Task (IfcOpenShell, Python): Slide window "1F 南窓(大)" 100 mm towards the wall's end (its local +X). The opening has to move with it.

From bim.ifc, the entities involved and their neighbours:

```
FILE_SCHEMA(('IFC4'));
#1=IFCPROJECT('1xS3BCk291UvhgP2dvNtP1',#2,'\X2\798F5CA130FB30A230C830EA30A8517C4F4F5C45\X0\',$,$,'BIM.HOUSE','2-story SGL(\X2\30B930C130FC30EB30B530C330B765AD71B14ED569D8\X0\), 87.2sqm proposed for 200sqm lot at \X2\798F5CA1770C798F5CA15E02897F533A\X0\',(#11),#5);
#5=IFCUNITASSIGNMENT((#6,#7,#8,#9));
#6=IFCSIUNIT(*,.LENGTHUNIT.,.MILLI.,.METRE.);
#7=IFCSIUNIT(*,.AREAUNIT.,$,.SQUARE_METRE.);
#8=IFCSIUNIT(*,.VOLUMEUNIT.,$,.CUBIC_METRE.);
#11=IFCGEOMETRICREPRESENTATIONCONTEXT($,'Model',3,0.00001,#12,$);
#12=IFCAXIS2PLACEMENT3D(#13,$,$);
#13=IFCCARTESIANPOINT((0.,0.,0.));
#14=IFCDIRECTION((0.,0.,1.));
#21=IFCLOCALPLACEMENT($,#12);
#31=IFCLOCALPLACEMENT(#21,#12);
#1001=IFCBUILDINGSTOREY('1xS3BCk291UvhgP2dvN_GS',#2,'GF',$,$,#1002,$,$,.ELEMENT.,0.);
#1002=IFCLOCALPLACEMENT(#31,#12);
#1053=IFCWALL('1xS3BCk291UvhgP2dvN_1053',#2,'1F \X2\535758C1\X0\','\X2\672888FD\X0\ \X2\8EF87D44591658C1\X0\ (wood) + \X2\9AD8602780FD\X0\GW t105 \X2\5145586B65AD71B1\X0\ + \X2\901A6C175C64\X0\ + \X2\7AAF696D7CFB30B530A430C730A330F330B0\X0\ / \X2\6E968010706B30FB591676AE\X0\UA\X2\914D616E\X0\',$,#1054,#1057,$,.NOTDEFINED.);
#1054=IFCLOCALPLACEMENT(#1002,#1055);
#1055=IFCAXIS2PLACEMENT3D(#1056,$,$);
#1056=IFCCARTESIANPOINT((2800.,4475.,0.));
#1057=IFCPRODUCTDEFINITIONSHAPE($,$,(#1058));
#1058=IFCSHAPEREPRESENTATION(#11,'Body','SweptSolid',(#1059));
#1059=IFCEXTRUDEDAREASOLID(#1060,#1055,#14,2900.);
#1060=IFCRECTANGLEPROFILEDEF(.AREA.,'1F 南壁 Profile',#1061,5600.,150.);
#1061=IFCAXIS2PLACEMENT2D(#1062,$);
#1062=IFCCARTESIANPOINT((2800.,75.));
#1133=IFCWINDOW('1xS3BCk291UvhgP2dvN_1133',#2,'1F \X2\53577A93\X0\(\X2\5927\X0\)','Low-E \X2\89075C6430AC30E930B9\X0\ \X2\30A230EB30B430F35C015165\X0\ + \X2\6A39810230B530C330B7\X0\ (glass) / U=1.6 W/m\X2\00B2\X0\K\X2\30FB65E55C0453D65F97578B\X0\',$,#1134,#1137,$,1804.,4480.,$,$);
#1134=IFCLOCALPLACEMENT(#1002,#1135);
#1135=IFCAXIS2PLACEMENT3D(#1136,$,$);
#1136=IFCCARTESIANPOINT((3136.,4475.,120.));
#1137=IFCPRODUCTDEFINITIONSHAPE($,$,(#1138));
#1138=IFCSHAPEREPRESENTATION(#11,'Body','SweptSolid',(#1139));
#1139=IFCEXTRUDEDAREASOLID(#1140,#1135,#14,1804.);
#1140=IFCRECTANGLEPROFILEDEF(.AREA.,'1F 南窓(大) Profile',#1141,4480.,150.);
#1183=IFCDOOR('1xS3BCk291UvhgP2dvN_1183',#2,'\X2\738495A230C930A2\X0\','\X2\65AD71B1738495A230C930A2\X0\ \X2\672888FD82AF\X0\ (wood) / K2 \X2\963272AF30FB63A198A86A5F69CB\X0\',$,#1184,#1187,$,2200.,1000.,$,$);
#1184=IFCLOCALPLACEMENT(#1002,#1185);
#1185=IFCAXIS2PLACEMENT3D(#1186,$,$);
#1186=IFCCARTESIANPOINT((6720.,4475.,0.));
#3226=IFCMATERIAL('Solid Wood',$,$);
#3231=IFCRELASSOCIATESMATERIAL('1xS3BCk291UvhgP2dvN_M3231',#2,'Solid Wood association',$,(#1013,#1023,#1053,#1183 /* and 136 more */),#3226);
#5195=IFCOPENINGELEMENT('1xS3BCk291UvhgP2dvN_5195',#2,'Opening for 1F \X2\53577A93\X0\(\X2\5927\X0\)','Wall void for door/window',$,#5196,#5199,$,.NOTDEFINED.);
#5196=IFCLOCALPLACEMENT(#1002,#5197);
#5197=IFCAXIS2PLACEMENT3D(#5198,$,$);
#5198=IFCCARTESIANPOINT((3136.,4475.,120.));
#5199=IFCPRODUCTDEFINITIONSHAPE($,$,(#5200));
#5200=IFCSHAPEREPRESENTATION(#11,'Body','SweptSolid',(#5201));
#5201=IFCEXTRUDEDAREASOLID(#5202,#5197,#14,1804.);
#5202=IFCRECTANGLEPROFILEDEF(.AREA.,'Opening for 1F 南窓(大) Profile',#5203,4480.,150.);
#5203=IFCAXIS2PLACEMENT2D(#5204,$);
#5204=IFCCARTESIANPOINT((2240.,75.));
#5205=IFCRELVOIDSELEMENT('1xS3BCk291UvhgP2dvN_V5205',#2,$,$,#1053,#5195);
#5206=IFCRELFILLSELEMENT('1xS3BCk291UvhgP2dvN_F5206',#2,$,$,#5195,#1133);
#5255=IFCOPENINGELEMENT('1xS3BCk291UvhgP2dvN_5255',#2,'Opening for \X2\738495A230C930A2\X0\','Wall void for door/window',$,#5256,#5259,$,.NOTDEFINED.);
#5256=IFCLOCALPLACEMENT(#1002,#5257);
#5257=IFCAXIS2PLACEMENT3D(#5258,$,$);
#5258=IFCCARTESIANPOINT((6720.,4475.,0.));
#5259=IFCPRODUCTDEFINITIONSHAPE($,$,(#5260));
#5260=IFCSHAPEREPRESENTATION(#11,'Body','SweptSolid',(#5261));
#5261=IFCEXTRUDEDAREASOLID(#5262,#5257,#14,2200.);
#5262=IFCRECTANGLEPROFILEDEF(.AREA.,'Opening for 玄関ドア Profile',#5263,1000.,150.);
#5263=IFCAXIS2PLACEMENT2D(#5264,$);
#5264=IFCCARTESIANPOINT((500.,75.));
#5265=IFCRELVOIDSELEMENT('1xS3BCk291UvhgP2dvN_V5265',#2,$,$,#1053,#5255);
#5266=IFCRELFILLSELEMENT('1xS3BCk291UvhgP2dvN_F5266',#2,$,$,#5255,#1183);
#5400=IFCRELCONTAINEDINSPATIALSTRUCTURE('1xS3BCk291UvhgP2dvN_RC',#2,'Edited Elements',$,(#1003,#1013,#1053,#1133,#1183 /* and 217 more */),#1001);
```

```python
import ifcopenshell
import ifcopenshell.api.geometry
import ifcopenshell.util.placement
import ifcopenshell.util.unit

model = ifcopenshell.open("bim.ifc")
unit_scale = ifcopenshell.util.unit.calculate_unit_scale(model)

window = model.by_guid("1xS3BCk291UvhgP2dvN_1133")
opening = window.FillsVoids[0].RelatingOpeningElement
wall = opening.VoidsElements[0].RelatingBuildingElement

wall_matrix = ifcopenshell.util.placement.get_local_placement(wall.ObjectPlacement)
shift = wall_matrix[:3, 0] * 0.1 / unit_scale
before = ifcopenshell.util.placement.get_local_placement(window.ObjectPlacement)[:3, 3].copy()

# The window is not placed relative to its opening, so move both.
for product in (opening, window):
    matrix = ifcopenshell.util.placement.get_local_placement(product.ObjectPlacement)
    matrix[:3, 3] += shift
    ifcopenshell.api.geometry.edit_object_placement(model, product=product, matrix=matrix, is_si=False)

after = ifcopenshell.util.placement.get_local_placement(window.ObjectPlacement)[:3, 3]
print("window moved by", (after - before).round(3) + 0.0)

model.write("bim_v2.ifc")
```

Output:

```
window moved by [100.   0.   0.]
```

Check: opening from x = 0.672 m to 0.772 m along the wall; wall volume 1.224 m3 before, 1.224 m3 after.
